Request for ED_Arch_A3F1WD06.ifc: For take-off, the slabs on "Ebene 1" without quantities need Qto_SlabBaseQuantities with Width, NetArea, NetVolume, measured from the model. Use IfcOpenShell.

First a look at what the model holds.

```python
import ifcopenshell
import ifcopenshell.util.element
import ifcopenshell.util.unit

model = ifcopenshell.open("ED_Arch_A3F1WD06.ifc")
print(model.schema)
for unit_type in ("LENGTHUNIT", "AREAUNIT", "VOLUMEUNIT"):
    print(unit_type, ifcopenshell.util.unit.calculate_unit_scale(model, unit_type))
storey = next(s for s in model.by_type("IfcBuildingStorey") if s.Name == "Ebene 1")
slabs = [e for e in ifcopenshell.util.element.get_decomposition(storey) if e.is_a("IfcSlab")]
for e in sorted(slabs, key=lambda e: e.id()):
    print(e.id(), e.is_a(), e.Name, list(ifcopenshell.util.element.get_psets(e, qtos_only=True)), sep=" | ")
```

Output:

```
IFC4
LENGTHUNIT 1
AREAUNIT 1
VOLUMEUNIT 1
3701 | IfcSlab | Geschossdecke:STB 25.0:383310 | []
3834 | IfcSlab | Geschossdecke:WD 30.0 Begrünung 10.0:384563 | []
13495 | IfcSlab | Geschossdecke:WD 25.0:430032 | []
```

```python
import ifcopenshell
import ifcopenshell.api.pset
import ifcopenshell.geom
import ifcopenshell.util.element
import ifcopenshell.util.shape
import ifcopenshell.util.unit

model = ifcopenshell.open("ED_Arch_A3F1WD06.ifc")
unit_scale = ifcopenshell.util.unit.calculate_unit_scale(model)
area_scale = ifcopenshell.util.unit.calculate_unit_scale(model, "AREAUNIT")
volume_scale = ifcopenshell.util.unit.calculate_unit_scale(model, "VOLUMEUNIT")
settings = ifcopenshell.geom.settings()

storey = next(s for s in model.by_type("IfcBuildingStorey") if s.Name == "Ebene 1")
slabs = [e for e in ifcopenshell.util.element.get_decomposition(storey) if e.is_a("IfcSlab")]

for e in sorted(slabs, key=lambda e: e.id()):
    if ifcopenshell.util.element.get_psets(e, qtos_only=True, should_inherit=False):
        continue
    # Geometry comes back in metres, in the element's own axes.
    shape = ifcopenshell.geom.create_shape(settings, e)
    values = {
        "Width": ifcopenshell.util.shape.get_z(shape.geometry) / unit_scale,
        "NetArea": ifcopenshell.util.shape.get_footprint_area(shape.geometry) / area_scale,
        "NetVolume": ifcopenshell.util.shape.get_volume(shape.geometry) / volume_scale,
    }
    qto = ifcopenshell.api.pset.add_qto(model, product=e, name="Qto_SlabBaseQuantities")
    ifcopenshell.api.pset.edit_qto(model, qto=qto, properties=values)
    print(e.id(), {k: round(v, 3) for k, v in values.items()})

model.write("ED_Arch_A3F1WD06-out.ifc")
```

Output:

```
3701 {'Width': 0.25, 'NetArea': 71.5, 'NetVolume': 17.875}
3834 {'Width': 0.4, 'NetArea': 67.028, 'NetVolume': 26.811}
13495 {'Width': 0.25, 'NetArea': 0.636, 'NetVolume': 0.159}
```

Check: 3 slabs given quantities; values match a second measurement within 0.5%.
